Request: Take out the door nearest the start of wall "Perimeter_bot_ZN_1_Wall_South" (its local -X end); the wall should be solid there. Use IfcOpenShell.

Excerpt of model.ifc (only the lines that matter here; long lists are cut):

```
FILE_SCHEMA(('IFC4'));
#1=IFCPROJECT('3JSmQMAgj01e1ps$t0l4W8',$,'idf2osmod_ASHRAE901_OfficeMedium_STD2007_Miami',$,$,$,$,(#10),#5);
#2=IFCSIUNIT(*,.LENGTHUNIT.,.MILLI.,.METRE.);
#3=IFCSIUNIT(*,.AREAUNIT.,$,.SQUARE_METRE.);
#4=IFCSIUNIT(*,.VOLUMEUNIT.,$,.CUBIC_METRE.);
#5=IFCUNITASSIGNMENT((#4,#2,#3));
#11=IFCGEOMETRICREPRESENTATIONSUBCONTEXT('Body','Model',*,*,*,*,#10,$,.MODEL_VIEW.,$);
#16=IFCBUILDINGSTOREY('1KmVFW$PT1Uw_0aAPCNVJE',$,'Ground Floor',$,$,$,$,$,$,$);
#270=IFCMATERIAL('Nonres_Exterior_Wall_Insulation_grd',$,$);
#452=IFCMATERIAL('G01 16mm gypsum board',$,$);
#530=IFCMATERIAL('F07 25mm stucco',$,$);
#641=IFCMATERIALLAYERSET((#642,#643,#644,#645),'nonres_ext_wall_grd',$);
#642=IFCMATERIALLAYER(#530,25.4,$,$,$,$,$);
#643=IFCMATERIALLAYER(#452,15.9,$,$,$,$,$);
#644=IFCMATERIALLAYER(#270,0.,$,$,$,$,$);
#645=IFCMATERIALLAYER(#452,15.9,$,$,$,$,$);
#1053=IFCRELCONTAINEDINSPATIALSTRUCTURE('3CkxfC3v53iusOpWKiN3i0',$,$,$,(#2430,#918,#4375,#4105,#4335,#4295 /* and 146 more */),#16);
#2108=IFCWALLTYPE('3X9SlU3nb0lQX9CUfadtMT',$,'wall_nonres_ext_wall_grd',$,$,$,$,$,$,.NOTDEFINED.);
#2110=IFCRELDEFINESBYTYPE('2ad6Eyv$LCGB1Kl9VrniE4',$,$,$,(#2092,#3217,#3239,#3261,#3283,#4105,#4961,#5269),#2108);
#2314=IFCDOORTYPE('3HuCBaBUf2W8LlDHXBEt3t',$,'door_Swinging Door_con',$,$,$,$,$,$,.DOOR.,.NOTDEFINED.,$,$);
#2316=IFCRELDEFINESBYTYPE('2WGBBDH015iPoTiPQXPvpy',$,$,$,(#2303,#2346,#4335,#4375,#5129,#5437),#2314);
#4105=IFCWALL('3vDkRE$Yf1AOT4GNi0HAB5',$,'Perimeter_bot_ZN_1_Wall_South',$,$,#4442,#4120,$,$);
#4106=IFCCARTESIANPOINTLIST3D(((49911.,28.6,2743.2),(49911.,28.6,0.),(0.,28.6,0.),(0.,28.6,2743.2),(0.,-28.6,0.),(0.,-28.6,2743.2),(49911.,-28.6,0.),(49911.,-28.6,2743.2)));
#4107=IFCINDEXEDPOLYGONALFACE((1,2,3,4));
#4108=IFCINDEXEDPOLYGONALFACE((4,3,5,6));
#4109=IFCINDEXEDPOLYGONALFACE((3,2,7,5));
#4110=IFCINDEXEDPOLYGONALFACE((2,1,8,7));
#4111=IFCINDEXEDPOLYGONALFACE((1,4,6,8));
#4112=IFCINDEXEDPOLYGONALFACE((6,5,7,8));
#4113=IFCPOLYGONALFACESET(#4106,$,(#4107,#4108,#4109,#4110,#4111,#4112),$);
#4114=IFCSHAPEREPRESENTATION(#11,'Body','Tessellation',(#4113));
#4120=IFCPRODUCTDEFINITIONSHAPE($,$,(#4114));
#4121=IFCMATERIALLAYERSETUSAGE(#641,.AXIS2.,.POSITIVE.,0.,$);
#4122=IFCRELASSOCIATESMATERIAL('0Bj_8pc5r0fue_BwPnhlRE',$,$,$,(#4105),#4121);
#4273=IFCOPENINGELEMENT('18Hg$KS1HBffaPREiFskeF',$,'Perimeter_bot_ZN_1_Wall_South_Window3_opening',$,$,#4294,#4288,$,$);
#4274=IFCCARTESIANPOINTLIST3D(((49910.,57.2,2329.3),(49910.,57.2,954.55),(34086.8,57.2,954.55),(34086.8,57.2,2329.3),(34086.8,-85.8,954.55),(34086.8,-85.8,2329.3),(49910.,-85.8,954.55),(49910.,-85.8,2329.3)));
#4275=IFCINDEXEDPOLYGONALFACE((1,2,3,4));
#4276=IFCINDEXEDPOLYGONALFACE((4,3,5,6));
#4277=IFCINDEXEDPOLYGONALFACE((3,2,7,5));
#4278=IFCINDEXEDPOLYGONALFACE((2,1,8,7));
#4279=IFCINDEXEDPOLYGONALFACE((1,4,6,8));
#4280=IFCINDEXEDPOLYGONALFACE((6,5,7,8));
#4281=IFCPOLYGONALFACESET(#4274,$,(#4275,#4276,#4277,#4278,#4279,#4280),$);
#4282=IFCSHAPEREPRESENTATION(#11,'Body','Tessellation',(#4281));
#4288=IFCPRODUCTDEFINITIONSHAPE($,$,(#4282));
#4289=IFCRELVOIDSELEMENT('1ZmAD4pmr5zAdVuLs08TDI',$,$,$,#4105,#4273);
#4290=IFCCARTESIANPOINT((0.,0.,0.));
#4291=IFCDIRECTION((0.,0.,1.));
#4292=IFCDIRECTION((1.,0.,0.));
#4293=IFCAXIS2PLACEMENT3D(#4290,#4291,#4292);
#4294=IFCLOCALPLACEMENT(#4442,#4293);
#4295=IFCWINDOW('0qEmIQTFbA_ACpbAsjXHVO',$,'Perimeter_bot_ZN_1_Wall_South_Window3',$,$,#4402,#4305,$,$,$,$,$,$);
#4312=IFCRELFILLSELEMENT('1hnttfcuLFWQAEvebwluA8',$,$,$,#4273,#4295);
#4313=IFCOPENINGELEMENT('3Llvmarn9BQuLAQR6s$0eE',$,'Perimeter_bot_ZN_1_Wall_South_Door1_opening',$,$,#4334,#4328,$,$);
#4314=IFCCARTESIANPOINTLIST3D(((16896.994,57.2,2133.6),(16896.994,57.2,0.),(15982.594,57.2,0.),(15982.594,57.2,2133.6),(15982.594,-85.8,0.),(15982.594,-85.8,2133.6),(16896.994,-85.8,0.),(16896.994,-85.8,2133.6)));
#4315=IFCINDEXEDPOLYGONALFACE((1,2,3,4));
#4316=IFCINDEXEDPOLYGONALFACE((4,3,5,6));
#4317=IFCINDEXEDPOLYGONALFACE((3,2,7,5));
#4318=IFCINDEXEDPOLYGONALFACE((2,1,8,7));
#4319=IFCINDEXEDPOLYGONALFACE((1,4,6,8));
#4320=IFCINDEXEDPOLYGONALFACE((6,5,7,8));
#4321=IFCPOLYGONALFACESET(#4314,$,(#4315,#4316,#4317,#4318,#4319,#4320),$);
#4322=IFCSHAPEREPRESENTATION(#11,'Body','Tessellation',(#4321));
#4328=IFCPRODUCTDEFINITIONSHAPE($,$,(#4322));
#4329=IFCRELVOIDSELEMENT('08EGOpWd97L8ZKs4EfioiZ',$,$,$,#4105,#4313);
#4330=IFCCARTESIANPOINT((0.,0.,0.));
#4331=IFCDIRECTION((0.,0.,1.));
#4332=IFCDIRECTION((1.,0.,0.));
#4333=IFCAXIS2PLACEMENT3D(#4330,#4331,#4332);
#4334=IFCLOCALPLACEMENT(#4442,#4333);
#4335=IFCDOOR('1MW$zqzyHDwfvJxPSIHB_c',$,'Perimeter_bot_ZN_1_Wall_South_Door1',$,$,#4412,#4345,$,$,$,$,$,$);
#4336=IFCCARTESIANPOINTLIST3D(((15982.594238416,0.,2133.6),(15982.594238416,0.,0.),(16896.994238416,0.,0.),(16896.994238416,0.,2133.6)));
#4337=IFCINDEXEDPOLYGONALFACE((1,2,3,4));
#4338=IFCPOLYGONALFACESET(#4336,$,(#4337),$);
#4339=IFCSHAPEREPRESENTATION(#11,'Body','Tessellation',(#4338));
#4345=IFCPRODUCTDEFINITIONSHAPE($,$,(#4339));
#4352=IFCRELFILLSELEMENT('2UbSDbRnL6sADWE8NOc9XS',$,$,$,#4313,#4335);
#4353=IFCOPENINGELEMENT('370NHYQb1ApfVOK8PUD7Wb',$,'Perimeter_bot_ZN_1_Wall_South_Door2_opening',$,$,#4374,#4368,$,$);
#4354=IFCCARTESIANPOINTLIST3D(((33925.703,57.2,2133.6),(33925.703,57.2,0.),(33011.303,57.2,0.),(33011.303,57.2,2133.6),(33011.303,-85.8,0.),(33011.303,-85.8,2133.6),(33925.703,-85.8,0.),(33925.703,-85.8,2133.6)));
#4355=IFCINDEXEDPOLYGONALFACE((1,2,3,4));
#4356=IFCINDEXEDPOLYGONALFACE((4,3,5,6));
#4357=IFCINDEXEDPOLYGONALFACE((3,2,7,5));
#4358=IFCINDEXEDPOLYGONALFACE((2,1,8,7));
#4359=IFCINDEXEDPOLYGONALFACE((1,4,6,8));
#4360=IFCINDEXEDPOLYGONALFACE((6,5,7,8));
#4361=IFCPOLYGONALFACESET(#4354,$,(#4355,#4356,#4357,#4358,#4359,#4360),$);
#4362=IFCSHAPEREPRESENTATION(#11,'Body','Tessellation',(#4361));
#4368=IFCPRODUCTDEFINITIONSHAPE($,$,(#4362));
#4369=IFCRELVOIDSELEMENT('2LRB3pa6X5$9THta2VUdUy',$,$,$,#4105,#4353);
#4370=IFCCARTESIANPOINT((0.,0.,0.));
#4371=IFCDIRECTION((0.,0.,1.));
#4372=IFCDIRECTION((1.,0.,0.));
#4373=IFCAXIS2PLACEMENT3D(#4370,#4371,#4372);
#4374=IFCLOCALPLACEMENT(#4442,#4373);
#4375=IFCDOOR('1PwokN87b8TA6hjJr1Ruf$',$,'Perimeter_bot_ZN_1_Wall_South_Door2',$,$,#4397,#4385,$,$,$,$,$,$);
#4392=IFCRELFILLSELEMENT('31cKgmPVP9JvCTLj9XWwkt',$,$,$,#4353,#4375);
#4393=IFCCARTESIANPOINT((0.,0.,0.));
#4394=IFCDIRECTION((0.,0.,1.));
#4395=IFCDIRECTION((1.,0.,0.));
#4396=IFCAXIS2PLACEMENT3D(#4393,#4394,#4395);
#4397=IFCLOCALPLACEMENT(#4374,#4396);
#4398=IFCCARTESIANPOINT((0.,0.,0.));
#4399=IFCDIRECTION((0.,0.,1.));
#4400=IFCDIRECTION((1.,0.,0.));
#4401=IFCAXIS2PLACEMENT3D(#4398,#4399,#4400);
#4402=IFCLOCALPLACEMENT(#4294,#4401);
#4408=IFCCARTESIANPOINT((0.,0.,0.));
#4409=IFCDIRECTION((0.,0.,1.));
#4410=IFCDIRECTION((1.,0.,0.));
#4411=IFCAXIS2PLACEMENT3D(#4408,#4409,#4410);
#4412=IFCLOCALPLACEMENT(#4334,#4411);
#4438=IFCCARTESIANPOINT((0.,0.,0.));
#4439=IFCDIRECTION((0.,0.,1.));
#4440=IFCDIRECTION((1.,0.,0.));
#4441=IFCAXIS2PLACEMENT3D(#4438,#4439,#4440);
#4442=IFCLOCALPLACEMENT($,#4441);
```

```python
import ifcopenshell
import ifcopenshell.api.feature
import ifcopenshell.api.root
import ifcopenshell.geom
import ifcopenshell.util.shape

model = ifcopenshell.open("model.ifc")
settings = ifcopenshell.geom.settings()


def volume(element):
    """Net volume in cubic metres, openings subtracted."""
    shape = ifcopenshell.geom.create_shape(settings, element)
    return ifcopenshell.util.shape.get_volume(shape.geometry)


door = model.by_guid("1MW$zqzyHDwfvJxPSIHB_c")
opening = door.FillsVoids[0].RelatingOpeningElement
wall = opening.VoidsElements[0].RelatingBuildingElement
before = volume(wall)

ifcopenshell.api.root.remove_product(model, product=door)
ifcopenshell.api.feature.remove_feature(model, feature=opening)

after = volume(wall)

print(f"wall volume {before:.3f} -> {after:.3f} m3")

model.write("model_rev.ifc")
```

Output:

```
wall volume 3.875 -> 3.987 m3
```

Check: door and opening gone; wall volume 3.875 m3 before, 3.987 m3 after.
